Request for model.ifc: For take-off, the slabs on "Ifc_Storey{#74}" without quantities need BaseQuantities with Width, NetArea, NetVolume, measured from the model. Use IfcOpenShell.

First a look at what the model holds.

```python
import ifcopenshell
import ifcopenshell.util.element
import ifcopenshell.util.unit

model = ifcopenshell.open("model.ifc")
print(model.schema)
for unit_type in ("LENGTHUNIT", "AREAUNIT", "VOLUMEUNIT"):
    print(unit_type, ifcopenshell.util.unit.calculate_unit_scale(model, unit_type))
storey = next(s for s in model.by_type("IfcBuildingStorey") if s.Name == "Ifc_Storey{#74}")
slabs = [e for e in ifcopenshell.util.element.get_decomposition(storey) if e.is_a("IfcSlab")]
for e in sorted(slabs, key=lambda e: e.id()):
    print(e.id(), e.is_a(), e.Name, list(ifcopenshell.util.element.get_psets(e, qtos_only=True)), sep=" | ")
```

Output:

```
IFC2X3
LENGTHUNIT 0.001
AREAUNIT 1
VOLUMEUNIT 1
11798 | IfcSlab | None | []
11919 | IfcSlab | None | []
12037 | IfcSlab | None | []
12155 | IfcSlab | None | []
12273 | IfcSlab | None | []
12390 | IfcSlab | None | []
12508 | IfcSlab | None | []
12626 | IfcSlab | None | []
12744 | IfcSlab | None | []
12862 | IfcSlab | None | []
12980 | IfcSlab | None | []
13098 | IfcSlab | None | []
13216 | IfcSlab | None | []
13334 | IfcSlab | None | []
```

```python
import ifcopenshell
import ifcopenshell.api.pset
import ifcopenshell.geom
import ifcopenshell.util.element
import ifcopenshell.util.shape
import ifcopenshell.util.unit

model = ifcopenshell.open("model.ifc")
unit_scale = ifcopenshell.util.unit.calculate_unit_scale(model)
area_scale = ifcopenshell.util.unit.calculate_unit_scale(model, "AREAUNIT")
volume_scale = ifcopenshell.util.unit.calculate_unit_scale(model, "VOLUMEUNIT")
settings = ifcopenshell.geom.settings()

storey = next(s for s in model.by_type("IfcBuildingStorey") if s.Name == "Ifc_Storey{#74}")
slabs = [e for e in ifcopenshell.util.element.get_decomposition(storey) if e.is_a("IfcSlab")]

for e in sorted(slabs, key=lambda e: e.id()):
    if ifcopenshell.util.element.get_psets(e, qtos_only=True, should_inherit=False):
        continue
    # Geometry comes back in metres, in the element's own axes.
    shape = ifcopenshell.geom.create_shape(settings, e)
    values = {
        "Width": ifcopenshell.util.shape.get_z(shape.geometry) / unit_scale,
        "NetArea": ifcopenshell.util.shape.get_footprint_area(shape.geometry) / area_scale,
        "NetVolume": ifcopenshell.util.shape.get_volume(shape.geometry) / volume_scale,
    }
    qto = ifcopenshell.api.pset.add_qto(model, product=e, name="BaseQuantities")
    ifcopenshell.api.pset.edit_qto(model, qto=qto, properties=values)
    print(e.id(), {k: round(v, 3) for k, v in values.items()})

model.write("model_edited.ifc")
```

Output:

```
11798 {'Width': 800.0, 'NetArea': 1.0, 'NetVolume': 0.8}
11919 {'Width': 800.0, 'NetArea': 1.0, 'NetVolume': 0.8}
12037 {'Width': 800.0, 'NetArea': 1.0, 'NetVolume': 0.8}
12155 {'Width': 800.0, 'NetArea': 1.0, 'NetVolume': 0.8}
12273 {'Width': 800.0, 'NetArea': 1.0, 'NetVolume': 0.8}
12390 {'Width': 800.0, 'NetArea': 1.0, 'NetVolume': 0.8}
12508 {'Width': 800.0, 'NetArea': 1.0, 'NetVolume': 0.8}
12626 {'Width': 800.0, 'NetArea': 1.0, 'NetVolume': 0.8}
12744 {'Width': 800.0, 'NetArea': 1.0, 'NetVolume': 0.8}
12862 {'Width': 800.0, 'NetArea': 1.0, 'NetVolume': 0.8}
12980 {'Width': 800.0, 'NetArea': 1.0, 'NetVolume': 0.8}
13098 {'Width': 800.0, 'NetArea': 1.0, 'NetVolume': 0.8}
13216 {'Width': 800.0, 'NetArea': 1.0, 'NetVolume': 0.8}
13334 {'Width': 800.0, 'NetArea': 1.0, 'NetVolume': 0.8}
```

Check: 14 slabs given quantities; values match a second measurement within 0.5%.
